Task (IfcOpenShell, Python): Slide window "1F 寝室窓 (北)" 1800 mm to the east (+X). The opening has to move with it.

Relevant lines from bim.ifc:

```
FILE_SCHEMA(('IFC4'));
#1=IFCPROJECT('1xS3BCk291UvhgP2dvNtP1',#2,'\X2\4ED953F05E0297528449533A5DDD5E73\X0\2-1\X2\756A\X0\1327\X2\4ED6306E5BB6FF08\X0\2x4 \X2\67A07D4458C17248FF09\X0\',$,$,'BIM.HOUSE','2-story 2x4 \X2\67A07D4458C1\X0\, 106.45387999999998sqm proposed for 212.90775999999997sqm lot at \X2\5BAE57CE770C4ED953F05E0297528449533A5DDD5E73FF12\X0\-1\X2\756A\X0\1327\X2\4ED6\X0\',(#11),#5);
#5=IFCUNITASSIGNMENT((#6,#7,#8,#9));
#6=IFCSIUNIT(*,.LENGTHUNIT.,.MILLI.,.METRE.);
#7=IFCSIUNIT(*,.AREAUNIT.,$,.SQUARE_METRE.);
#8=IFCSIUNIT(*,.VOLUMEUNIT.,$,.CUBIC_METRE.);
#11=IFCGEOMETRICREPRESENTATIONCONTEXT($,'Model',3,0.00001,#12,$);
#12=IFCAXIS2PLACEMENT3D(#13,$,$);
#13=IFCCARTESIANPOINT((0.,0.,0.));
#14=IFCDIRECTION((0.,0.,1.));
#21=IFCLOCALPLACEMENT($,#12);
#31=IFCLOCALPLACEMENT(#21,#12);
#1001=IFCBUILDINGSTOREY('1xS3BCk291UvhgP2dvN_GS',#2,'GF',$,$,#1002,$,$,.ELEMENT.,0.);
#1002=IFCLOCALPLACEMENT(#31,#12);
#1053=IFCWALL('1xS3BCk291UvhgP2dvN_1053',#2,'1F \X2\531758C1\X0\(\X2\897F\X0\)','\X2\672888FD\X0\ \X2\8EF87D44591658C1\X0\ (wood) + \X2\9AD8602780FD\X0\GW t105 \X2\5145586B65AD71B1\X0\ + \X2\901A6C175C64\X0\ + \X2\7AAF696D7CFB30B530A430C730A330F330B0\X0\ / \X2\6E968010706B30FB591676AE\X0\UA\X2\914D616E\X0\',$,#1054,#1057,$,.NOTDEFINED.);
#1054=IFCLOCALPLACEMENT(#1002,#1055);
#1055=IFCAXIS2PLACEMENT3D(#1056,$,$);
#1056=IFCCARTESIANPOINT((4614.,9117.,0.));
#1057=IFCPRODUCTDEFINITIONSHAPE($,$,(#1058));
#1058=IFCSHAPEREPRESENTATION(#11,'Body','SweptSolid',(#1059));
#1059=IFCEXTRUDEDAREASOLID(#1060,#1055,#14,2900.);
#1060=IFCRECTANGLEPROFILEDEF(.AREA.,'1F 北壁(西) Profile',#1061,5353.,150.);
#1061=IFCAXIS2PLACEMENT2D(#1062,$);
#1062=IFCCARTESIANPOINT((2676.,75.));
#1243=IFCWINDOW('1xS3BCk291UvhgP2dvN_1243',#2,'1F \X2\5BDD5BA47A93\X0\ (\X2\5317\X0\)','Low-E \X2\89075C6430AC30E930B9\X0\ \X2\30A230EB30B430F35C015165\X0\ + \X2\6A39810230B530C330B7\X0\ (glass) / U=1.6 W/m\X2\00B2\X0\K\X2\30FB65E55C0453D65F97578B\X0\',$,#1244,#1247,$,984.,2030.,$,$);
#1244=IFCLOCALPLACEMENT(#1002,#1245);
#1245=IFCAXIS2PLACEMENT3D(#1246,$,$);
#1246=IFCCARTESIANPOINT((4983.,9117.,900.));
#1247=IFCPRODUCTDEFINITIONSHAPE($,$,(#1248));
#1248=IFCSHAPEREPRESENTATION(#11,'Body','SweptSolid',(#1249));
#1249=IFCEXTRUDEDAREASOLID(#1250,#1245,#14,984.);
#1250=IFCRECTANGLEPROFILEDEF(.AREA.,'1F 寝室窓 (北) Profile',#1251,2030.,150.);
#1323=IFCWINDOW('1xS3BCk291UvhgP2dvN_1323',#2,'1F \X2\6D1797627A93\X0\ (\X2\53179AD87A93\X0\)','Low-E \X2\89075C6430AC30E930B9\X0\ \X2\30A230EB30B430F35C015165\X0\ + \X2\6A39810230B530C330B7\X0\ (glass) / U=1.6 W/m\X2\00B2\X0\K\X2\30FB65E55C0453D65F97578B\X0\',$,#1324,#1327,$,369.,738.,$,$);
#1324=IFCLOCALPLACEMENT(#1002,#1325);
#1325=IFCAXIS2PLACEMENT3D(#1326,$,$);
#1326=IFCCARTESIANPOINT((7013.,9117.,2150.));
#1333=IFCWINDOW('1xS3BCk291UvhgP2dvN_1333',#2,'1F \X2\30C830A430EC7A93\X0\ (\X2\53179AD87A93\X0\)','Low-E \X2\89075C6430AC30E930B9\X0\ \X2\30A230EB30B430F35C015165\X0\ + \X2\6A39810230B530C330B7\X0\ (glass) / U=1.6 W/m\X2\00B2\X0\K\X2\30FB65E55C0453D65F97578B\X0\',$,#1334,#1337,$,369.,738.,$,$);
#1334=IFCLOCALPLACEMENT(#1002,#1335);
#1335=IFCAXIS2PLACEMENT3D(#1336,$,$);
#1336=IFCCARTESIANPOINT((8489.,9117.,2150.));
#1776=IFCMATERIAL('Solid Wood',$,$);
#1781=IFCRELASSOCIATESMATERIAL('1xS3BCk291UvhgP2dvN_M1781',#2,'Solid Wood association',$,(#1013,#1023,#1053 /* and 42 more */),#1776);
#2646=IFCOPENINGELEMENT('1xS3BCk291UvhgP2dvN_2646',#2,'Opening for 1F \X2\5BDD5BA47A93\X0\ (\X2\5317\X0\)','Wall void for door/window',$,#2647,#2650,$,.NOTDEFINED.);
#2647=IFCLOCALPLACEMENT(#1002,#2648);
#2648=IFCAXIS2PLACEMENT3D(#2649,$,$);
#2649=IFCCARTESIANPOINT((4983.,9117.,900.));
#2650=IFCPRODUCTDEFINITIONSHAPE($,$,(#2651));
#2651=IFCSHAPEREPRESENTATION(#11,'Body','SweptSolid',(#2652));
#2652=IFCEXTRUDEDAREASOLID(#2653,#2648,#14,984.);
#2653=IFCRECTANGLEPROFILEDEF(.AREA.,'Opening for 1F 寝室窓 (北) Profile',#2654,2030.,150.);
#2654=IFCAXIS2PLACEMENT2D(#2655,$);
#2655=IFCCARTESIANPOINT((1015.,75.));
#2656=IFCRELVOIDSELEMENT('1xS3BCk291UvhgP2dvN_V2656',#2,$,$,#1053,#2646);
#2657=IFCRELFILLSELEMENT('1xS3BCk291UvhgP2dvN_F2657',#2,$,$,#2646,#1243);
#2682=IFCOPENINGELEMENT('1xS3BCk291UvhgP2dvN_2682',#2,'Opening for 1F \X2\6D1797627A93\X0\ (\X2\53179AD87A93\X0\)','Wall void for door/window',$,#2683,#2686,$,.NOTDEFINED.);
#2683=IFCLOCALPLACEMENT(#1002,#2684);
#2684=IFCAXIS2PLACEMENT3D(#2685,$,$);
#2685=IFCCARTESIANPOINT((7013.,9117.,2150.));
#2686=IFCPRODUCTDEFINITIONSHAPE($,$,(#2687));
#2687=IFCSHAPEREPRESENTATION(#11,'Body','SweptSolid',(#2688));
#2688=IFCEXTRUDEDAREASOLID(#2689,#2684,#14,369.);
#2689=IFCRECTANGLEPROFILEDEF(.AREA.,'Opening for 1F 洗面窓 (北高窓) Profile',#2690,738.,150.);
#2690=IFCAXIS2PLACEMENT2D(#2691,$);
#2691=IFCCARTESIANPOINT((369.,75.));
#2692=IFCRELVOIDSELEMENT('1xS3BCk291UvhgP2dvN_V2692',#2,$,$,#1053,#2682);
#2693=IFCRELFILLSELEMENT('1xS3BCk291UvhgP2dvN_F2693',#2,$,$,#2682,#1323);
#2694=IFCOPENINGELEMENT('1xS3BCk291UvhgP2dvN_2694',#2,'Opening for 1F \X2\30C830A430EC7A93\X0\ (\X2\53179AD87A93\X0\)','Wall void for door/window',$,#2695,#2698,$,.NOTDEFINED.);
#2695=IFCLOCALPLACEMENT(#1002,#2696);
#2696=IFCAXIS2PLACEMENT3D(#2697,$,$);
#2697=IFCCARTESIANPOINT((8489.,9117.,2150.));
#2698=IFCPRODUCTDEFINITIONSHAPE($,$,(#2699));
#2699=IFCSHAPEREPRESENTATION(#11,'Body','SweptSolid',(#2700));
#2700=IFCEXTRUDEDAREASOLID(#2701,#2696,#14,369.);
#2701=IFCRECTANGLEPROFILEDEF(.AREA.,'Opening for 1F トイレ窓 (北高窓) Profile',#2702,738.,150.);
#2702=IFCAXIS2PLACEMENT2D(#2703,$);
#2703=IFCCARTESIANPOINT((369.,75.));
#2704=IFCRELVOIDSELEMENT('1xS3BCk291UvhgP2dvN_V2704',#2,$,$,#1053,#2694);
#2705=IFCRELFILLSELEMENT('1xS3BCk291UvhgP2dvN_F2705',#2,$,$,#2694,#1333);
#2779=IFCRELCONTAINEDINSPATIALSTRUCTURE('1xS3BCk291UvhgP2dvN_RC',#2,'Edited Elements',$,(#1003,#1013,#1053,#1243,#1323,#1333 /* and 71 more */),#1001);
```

```python
import ifcopenshell
import ifcopenshell.api.geometry
import ifcopenshell.util.placement

model = ifcopenshell.open("bim.ifc")

window = model.by_guid("1xS3BCk291UvhgP2dvN_1243")
opening = window.FillsVoids[0].RelatingOpeningElement
wall = opening.VoidsElements[0].RelatingBuildingElement

wall_matrix = ifcopenshell.util.placement.get_local_placement(wall.ObjectPlacement)
shift = wall_matrix[:3, 0] * 1800.0
before = ifcopenshell.util.placement.get_local_placement(window.ObjectPlacement)[:3, 3].copy()

# The window is not placed relative to its opening, so move both.
for product in (opening, window):
    matrix = ifcopenshell.util.placement.get_local_placement(product.ObjectPlacement)
    matrix[:3, 3] += shift
    ifcopenshell.api.geometry.edit_object_placement(model, product=product, matrix=matrix, is_si=False)

after = ifcopenshell.util.placement.get_local_placement(window.ObjectPlacement)[:3, 3]
print("window moved by", (after - before).round(3) + 0.0)

model.write("bim_rev.ifc")
```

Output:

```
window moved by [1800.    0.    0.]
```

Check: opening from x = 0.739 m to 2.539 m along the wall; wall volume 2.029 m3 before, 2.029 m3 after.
